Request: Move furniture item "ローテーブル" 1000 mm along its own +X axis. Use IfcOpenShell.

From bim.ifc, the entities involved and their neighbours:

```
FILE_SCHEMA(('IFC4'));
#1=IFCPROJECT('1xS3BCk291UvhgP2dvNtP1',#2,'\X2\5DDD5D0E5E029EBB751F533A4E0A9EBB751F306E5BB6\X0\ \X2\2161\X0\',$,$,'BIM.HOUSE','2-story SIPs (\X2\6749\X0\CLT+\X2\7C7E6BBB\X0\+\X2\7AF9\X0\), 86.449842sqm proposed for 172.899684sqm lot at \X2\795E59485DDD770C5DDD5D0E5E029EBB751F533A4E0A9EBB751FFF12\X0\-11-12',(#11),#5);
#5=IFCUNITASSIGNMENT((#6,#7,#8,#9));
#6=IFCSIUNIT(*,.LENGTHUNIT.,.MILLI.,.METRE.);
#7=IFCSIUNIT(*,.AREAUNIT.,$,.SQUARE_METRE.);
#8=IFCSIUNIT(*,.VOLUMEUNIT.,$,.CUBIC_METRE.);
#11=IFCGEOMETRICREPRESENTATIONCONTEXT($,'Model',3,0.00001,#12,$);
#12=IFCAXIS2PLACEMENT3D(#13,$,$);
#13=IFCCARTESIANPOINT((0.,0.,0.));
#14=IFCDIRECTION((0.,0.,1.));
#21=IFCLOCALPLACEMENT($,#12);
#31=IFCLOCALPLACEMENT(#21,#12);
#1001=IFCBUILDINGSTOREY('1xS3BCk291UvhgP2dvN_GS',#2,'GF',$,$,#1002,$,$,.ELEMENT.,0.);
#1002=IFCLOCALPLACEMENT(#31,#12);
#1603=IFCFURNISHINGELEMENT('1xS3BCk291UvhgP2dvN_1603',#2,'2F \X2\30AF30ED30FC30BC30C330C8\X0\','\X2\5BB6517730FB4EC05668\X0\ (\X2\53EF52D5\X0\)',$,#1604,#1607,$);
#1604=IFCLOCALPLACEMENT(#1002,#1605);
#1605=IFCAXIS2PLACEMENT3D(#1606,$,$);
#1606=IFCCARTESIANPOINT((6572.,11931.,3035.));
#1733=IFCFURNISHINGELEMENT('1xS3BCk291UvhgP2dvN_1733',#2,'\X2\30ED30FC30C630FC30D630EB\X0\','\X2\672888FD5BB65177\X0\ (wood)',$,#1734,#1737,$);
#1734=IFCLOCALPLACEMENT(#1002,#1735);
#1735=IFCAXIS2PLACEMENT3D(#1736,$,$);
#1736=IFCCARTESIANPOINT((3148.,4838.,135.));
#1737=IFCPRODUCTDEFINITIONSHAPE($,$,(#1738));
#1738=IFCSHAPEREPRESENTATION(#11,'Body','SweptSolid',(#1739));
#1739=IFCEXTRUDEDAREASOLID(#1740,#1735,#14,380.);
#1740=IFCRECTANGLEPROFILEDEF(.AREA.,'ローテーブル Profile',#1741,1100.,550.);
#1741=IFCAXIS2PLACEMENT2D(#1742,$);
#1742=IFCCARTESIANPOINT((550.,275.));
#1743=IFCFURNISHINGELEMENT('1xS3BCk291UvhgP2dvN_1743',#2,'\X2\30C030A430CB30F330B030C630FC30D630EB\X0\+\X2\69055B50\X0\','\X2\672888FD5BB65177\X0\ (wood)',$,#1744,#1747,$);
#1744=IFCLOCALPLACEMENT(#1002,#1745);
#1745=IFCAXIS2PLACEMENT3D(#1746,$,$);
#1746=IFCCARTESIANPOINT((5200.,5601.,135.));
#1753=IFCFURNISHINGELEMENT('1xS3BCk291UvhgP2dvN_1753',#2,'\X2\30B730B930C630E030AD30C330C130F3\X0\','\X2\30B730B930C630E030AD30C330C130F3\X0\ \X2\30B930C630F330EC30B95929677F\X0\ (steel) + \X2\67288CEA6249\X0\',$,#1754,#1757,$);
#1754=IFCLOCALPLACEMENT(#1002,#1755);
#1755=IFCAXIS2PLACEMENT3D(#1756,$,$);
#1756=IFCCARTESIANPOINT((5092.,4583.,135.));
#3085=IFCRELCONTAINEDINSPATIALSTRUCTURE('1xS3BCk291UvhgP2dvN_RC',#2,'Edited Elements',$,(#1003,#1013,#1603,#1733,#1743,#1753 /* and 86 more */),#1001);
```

```python
import ifcopenshell
import ifcopenshell.api.geometry
import ifcopenshell.util.placement

model = ifcopenshell.open("bim.ifc")

item = model.by_guid("1xS3BCk291UvhgP2dvN_1733")
matrix = ifcopenshell.util.placement.get_local_placement(item.ObjectPlacement)
matrix[:3, 3] += matrix[:3, 0] * 1000.0
ifcopenshell.api.geometry.edit_object_placement(model, product=item, matrix=matrix, is_si=False)

print(ifcopenshell.util.placement.get_local_placement(item.ObjectPlacement).round(3) + 0.0)

model.write("bim_updated.ifc")
```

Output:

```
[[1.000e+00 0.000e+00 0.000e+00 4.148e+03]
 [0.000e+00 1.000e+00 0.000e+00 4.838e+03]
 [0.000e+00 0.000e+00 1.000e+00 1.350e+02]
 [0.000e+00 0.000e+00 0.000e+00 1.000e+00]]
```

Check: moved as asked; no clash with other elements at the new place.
